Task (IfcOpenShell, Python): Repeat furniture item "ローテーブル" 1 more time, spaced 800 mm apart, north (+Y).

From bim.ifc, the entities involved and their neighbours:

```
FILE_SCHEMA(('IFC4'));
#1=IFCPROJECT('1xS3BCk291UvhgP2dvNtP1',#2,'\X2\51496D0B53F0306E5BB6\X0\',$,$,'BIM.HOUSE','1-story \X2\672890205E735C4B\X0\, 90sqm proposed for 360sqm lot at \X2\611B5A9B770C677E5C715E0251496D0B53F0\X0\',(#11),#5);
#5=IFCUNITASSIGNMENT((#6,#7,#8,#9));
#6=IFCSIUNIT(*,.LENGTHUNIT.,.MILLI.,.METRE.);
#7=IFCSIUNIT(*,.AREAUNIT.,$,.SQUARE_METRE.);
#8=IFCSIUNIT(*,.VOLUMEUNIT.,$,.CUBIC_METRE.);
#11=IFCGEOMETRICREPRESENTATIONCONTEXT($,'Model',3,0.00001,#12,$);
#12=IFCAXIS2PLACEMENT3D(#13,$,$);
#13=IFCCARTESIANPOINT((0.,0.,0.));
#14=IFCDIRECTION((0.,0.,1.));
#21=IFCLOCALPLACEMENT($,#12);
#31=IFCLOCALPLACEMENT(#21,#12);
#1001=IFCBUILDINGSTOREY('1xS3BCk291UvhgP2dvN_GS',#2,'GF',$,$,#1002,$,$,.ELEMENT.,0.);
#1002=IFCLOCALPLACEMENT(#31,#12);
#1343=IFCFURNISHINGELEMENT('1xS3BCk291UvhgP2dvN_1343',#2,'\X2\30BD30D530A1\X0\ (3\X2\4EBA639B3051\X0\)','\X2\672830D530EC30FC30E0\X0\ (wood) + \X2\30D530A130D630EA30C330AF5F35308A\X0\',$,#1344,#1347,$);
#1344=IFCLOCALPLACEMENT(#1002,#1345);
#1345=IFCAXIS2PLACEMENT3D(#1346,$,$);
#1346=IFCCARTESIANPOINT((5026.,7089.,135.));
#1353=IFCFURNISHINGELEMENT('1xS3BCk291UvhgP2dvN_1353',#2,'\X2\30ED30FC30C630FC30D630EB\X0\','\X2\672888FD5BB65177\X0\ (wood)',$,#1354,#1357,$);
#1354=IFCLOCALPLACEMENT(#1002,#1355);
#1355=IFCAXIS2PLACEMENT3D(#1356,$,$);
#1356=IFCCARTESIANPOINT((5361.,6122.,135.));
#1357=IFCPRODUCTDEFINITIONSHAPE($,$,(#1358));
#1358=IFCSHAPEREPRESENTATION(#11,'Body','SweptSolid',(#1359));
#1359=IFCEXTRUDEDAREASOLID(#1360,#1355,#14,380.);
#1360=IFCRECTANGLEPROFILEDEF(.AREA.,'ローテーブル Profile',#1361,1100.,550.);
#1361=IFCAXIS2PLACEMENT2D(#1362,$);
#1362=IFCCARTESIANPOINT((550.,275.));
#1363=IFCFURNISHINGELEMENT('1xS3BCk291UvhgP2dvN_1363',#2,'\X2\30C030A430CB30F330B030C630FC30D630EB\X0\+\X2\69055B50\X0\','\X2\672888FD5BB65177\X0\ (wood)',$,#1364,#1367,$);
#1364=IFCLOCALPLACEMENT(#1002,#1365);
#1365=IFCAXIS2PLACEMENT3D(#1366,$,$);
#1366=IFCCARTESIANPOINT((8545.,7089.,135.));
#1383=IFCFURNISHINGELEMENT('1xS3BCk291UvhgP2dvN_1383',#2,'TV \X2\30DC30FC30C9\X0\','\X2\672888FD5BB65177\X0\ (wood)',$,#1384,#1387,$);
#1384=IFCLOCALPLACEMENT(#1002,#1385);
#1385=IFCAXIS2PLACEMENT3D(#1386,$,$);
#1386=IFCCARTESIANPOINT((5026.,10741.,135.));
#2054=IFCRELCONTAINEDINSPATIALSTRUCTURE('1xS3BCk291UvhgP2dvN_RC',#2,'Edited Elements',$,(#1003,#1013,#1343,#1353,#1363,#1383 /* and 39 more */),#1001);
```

```python
import numpy as np
import ifcopenshell
import ifcopenshell.api.geometry
import ifcopenshell.api.root
import ifcopenshell.util.element
import ifcopenshell.util.placement
import ifcopenshell.util.unit

model = ifcopenshell.open("bim.ifc")
unit_scale = ifcopenshell.util.unit.calculate_unit_scale(model)


def reuse_history(source, copy):
    """copy_class also copies each property set's owner history, people and application; keep the originals."""
    for rel in copy.IsDefinedBy:
        if rel.is_a("IfcRelDefinesByProperties") and (history := rel.RelatingPropertyDefinition.OwnerHistory):
            rel.RelatingPropertyDefinition.OwnerHistory = source.OwnerHistory
            ifcopenshell.util.element.remove_deep2(model, history)


source = model.by_id(1353)
base = ifcopenshell.util.placement.get_local_placement(source.ObjectPlacement)
step = np.array([0.0, 1.0, 0.0]) * 0.8 / unit_scale

for i in range(1, 2):
    copy = ifcopenshell.api.root.copy_class(model, product=source)
    copy.Representation = ifcopenshell.util.element.copy_deep(
        model, source.Representation, exclude=["IfcGeometricRepresentationContext", "IfcRepresentationMap"]
    )
    reuse_history(source, copy)
    matrix = base.copy()
    matrix[:3, 3] += i * step
    print("added at", matrix[:3, 3].round(3) + 0.0)
    ifcopenshell.api.geometry.edit_object_placement(model, product=copy, matrix=matrix, is_si=False)

model.write("bim_rev.ifc")
```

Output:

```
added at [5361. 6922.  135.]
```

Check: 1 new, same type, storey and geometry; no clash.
